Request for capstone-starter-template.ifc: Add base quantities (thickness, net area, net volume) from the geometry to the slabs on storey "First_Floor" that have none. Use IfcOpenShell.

First a look at what the model holds.

```python
import ifcopenshell
import ifcopenshell.util.element
import ifcopenshell.util.unit

model = ifcopenshell.open("capstone-starter-template.ifc")
print(model.schema)
for unit_type in ("LENGTHUNIT", "AREAUNIT", "VOLUMEUNIT"):
    print(unit_type, ifcopenshell.util.unit.calculate_unit_scale(model, unit_type))
storey = next(s for s in model.by_type("IfcBuildingStorey") if s.Name == "First_Floor")
slabs = [e for e in ifcopenshell.util.element.get_decomposition(storey) if e.is_a("IfcSlab")]
for e in sorted(slabs, key=lambda e: e.id()):
    print(e.id(), e.is_a(), e.Name, list(ifcopenshell.util.element.get_psets(e, qtos_only=True)), sep=" | ")
```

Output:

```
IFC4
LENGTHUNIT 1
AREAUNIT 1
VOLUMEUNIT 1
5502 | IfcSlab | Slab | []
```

```python
import ifcopenshell
import ifcopenshell.api.pset
import ifcopenshell.geom
import ifcopenshell.util.element
import ifcopenshell.util.shape
import ifcopenshell.util.unit

model = ifcopenshell.open("capstone-starter-template.ifc")
unit_scale = ifcopenshell.util.unit.calculate_unit_scale(model)
area_scale = ifcopenshell.util.unit.calculate_unit_scale(model, "AREAUNIT")
volume_scale = ifcopenshell.util.unit.calculate_unit_scale(model, "VOLUMEUNIT")
settings = ifcopenshell.geom.settings()

storey = next(s for s in model.by_type("IfcBuildingStorey") if s.Name == "First_Floor")
slabs = [e for e in ifcopenshell.util.element.get_decomposition(storey) if e.is_a("IfcSlab")]

for e in sorted(slabs, key=lambda e: e.id()):
    if ifcopenshell.util.element.get_psets(e, qtos_only=True, should_inherit=False):
        continue
    # Geometry comes back in metres, in the element's own axes.
    shape = ifcopenshell.geom.create_shape(settings, e)
    values = {
        "Width": ifcopenshell.util.shape.get_z(shape.geometry) / unit_scale,
        "NetArea": ifcopenshell.util.shape.get_footprint_area(shape.geometry) / area_scale,
        "NetVolume": ifcopenshell.util.shape.get_volume(shape.geometry) / volume_scale,
    }
    qto = ifcopenshell.api.pset.add_qto(model, product=e, name="Qto_SlabBaseQuantities")
    ifcopenshell.api.pset.edit_qto(model, qto=qto, properties=values)
    print(e.id(), {k: round(v, 3) for k, v in values.items()})

model.write("capstone-starter-template_edited.ifc")
```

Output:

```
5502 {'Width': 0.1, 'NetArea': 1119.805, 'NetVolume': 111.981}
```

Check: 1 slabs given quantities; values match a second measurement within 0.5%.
